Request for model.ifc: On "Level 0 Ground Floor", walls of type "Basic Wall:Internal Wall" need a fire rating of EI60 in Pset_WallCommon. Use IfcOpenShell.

First a look at what the model holds.

```python
import ifcopenshell
import ifcopenshell.util.element

model = ifcopenshell.open("model.ifc")
print(model.schema)
storey = next(s for s in model.by_type("IfcBuildingStorey") if s.Name == "Level 0 Ground Floor")
walls = [e for e in ifcopenshell.util.element.get_decomposition(storey) if e.is_a("IfcWall")]
seen = {}
for e in walls:
    element_type = ifcopenshell.util.element.get_type(e)
    key = (element_type.Name if element_type != e and element_type else None, ifcopenshell.util.element.get_pset(e, "Pset_WallCommon", "FireRating"))
    seen[key] = seen.get(key, 0) + 1
for (name, value), count in sorted(seen.items(), key=str):
    print(count, "x", name, "|", value)
```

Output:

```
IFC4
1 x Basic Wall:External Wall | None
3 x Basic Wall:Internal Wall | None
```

```python
import ifcopenshell
import ifcopenshell.api.pset
import ifcopenshell.util.element

model = ifcopenshell.open("model.ifc")

storey = next(s for s in model.by_type("IfcBuildingStorey") if s.Name == "Level 0 Ground Floor")
walls = [e for e in ifcopenshell.util.element.get_decomposition(storey) if e.is_a("IfcWall")]

count = 0
for e in walls:
    element_type = ifcopenshell.util.element.get_type(e)
    if element_type in (None, e) or element_type.Name != "Basic Wall:Internal Wall":
        continue
    # add_pset returns the element's existing set when there is one.
    pset = ifcopenshell.api.pset.add_pset(model, product=e, name="Pset_WallCommon")
    ifcopenshell.api.pset.edit_pset(model, pset=pset, properties={"FireRating": "EI60"})
    count += 1

print(count, "walls updated")

model.write("model_rev.ifc")
```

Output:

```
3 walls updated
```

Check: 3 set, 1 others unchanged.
